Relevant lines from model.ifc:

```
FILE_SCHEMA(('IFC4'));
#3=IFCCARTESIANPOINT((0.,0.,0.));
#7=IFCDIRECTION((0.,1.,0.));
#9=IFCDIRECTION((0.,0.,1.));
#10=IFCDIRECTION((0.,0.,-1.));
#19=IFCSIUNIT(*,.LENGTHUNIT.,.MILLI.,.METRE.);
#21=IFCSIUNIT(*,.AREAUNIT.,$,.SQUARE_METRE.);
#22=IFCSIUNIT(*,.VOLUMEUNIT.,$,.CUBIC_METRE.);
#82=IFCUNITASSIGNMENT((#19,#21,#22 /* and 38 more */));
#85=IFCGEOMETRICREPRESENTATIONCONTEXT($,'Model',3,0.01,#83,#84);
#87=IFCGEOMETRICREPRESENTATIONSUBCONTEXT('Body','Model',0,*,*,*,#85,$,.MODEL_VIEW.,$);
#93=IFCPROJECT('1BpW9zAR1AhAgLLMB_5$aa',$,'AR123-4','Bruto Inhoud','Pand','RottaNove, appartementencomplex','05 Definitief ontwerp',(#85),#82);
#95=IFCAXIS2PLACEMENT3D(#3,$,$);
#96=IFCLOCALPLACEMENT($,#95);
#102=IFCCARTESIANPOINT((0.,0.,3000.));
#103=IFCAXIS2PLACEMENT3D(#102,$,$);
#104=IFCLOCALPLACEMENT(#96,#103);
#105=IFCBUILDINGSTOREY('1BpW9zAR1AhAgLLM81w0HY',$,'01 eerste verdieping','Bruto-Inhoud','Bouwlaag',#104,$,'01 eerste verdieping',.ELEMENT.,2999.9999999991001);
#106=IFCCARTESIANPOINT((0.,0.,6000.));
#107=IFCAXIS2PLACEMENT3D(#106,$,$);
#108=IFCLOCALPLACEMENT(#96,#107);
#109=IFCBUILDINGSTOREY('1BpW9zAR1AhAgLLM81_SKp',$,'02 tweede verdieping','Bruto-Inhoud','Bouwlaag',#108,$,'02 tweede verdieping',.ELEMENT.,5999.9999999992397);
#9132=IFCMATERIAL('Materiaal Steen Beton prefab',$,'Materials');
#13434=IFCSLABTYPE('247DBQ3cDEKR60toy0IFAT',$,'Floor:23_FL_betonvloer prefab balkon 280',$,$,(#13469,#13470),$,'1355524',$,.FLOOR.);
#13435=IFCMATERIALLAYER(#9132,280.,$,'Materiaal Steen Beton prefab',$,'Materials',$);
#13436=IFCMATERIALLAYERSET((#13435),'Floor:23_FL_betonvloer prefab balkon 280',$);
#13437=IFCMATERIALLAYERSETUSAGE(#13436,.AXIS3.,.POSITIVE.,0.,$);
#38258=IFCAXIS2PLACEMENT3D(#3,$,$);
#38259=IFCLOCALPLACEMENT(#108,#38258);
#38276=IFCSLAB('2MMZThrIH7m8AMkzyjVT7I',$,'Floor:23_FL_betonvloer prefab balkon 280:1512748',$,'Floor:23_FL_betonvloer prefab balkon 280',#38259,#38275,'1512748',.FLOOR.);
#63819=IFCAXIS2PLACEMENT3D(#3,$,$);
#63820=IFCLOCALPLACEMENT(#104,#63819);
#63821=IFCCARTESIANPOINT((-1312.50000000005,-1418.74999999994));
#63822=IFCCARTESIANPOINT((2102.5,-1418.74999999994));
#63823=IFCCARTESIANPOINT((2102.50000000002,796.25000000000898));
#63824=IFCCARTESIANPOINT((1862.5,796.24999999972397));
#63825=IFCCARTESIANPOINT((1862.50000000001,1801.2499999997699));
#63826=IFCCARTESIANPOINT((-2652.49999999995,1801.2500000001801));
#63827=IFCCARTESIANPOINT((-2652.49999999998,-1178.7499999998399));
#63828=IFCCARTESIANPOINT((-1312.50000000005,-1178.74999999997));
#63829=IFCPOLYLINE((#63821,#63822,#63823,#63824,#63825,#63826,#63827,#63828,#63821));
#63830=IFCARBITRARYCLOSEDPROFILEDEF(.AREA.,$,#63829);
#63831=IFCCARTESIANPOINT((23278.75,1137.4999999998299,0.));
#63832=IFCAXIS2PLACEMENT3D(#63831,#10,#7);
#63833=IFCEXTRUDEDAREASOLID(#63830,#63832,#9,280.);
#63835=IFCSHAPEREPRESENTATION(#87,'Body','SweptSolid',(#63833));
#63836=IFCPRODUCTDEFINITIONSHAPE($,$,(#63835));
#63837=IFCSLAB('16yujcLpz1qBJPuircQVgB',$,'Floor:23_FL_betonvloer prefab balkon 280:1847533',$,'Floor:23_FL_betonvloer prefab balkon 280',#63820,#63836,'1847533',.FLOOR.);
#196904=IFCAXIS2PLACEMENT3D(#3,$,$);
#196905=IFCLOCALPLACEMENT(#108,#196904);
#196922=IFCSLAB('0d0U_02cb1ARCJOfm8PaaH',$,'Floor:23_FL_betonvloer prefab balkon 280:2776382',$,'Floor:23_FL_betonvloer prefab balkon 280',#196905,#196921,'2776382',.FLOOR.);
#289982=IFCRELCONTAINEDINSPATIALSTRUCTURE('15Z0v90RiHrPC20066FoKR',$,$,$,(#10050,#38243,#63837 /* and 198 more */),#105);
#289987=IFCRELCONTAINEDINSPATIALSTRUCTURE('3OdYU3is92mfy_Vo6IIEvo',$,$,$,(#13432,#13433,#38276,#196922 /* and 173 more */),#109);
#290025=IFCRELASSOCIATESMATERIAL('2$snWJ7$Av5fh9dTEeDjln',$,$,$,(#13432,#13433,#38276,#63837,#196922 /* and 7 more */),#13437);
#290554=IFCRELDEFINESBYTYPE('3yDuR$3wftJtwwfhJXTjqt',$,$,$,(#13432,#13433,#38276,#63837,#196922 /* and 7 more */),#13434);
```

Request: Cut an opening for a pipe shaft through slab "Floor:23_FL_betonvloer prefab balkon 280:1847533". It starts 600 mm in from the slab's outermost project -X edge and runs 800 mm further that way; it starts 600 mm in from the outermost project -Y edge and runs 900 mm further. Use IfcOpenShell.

```python
import numpy as np
import ifcopenshell
import ifcopenshell.api.feature
import ifcopenshell.api.geometry
import ifcopenshell.api.root
import ifcopenshell.geom
import ifcopenshell.util.placement
import ifcopenshell.util.representation
import ifcopenshell.util.shape
import ifcopenshell.util.unit

model = ifcopenshell.open("model.ifc")
unit_scale = ifcopenshell.util.unit.calculate_unit_scale(model)
settings = ifcopenshell.geom.settings()


def volume(element):
    """Net volume in cubic metres, openings subtracted."""
    shape = ifcopenshell.geom.create_shape(settings, element)
    return ifcopenshell.util.shape.get_volume(shape.geometry)


slab = model.by_guid("16yujcLpz1qBJPuircQVgB")
before = volume(slab)

# Extent in the slab's own axes, in metres. The edges named are its -X and -Y sides.
slab_shape = ifcopenshell.geom.create_shape(settings, slab)
vertices = ifcopenshell.util.shape.get_vertices(slab_shape.geometry)
x_min, y_min, bottom = vertices.min(axis=0)
top = vertices[:, 2].max()

opening = ifcopenshell.api.root.create_entity(model, ifc_class="IfcOpeningElement", name="Pipe shaft opening", predefined_type="OPENING")
context = ifcopenshell.util.representation.get_context(model, "Model", "Body", "MODEL_VIEW")
width, depth = 0.8, 0.9
outline = [(0.0, 0.0), (width, 0.0), (width, depth), (0.0, depth), (0.0, 0.0)]
# Overshoot both faces by 50 mm so the cut is clean.
shape = ifcopenshell.api.geometry.add_slab_representation(
    model, context=context, depth=top - bottom + 0.1, polyline=outline
)
ifcopenshell.api.geometry.assign_representation(model, product=opening, representation=shape)

matrix = ifcopenshell.util.placement.get_local_placement(slab.ObjectPlacement)
matrix[:, 3] = matrix @ np.append(np.array([x_min + 0.6, y_min + 0.6, bottom - 0.05]) / unit_scale, 1.0)
ifcopenshell.api.geometry.edit_object_placement(model, product=opening, matrix=matrix, is_si=False)
ifcopenshell.api.feature.add_feature(model, feature=opening, element=slab)

after = volume(slab)

print(f"slab volume {before:.3f} -> {after:.3f} m3")

model.write("model_v2.ifc")
```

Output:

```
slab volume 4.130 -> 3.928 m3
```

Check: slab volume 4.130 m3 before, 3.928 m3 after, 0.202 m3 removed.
